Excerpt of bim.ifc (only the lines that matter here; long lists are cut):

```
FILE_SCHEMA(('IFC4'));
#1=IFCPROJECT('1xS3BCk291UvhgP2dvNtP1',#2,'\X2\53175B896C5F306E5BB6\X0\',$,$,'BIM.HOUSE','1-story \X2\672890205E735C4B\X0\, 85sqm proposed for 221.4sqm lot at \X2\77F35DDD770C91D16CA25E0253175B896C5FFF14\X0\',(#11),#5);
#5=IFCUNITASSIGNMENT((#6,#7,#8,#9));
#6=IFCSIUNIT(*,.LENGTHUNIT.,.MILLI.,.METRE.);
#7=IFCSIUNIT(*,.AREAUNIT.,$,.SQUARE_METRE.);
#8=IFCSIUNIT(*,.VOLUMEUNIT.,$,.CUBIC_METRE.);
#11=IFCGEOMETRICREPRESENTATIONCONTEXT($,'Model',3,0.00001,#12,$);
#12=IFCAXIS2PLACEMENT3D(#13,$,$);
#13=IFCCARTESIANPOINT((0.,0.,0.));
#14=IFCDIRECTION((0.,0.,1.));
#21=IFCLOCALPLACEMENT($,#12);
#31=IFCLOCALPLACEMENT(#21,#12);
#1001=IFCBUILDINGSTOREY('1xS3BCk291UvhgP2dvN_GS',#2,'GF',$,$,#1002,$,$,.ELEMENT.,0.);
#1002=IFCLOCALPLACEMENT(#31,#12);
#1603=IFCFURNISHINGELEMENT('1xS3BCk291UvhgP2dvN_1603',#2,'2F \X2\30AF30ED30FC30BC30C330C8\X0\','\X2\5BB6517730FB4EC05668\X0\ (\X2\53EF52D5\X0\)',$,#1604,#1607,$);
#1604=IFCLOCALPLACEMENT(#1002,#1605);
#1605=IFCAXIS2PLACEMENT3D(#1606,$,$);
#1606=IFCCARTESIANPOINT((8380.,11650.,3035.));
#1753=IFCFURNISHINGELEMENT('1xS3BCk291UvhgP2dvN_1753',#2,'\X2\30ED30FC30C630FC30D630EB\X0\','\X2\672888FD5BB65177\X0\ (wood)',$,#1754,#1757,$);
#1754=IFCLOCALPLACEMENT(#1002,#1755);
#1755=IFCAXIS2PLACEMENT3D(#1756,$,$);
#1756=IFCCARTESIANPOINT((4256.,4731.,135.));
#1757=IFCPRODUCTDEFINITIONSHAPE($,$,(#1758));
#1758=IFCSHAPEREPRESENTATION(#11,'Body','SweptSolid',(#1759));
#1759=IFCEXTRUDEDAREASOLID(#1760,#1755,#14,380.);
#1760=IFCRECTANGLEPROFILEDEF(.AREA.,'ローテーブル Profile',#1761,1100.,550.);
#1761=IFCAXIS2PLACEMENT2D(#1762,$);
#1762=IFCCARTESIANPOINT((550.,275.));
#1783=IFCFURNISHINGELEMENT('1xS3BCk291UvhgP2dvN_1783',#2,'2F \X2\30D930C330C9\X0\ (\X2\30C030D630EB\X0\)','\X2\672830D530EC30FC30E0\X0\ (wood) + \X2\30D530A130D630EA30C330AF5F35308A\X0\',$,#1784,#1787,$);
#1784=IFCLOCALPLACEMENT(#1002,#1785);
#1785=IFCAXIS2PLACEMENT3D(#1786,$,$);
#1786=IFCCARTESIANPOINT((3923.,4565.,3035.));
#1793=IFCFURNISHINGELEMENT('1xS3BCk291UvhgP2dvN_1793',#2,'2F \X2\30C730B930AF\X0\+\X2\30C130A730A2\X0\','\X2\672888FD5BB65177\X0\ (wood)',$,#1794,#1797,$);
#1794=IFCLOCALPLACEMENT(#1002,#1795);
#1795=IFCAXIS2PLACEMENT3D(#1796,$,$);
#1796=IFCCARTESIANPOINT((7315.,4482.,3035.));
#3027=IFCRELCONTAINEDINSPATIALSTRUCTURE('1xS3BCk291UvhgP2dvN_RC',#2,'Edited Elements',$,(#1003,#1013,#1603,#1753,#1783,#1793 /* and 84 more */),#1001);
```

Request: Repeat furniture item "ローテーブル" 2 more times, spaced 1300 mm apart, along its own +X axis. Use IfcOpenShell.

```python
import ifcopenshell
import ifcopenshell.api.geometry
import ifcopenshell.api.root
import ifcopenshell.util.element
import ifcopenshell.util.placement

model = ifcopenshell.open("bim.ifc")


def reuse_history(source, copy):
    """copy_class also copies each property set's owner history, people and application; keep the originals."""
    for rel in copy.IsDefinedBy:
        if rel.is_a("IfcRelDefinesByProperties") and (history := rel.RelatingPropertyDefinition.OwnerHistory):
            rel.RelatingPropertyDefinition.OwnerHistory = source.OwnerHistory
            ifcopenshell.util.element.remove_deep2(model, history)


source = model.by_guid("1xS3BCk291UvhgP2dvN_1753")
base = ifcopenshell.util.placement.get_local_placement(source.ObjectPlacement)
step = base[:3, 0] * 1300.0

for i in range(1, 3):
    copy = ifcopenshell.api.root.copy_class(model, product=source)
    copy.Representation = ifcopenshell.util.element.copy_deep(
        model, source.Representation, exclude=["IfcGeometricRepresentationContext", "IfcRepresentationMap"]
    )
    reuse_history(source, copy)
    matrix = base.copy()
    matrix[:3, 3] += i * step
    print("added at", matrix[:3, 3].round(3) + 0.0)
    ifcopenshell.api.geometry.edit_object_placement(model, product=copy, matrix=matrix, is_si=False)

model.write("bim_v2.ifc")
```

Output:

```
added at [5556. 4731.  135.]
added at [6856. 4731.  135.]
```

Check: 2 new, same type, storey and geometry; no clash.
